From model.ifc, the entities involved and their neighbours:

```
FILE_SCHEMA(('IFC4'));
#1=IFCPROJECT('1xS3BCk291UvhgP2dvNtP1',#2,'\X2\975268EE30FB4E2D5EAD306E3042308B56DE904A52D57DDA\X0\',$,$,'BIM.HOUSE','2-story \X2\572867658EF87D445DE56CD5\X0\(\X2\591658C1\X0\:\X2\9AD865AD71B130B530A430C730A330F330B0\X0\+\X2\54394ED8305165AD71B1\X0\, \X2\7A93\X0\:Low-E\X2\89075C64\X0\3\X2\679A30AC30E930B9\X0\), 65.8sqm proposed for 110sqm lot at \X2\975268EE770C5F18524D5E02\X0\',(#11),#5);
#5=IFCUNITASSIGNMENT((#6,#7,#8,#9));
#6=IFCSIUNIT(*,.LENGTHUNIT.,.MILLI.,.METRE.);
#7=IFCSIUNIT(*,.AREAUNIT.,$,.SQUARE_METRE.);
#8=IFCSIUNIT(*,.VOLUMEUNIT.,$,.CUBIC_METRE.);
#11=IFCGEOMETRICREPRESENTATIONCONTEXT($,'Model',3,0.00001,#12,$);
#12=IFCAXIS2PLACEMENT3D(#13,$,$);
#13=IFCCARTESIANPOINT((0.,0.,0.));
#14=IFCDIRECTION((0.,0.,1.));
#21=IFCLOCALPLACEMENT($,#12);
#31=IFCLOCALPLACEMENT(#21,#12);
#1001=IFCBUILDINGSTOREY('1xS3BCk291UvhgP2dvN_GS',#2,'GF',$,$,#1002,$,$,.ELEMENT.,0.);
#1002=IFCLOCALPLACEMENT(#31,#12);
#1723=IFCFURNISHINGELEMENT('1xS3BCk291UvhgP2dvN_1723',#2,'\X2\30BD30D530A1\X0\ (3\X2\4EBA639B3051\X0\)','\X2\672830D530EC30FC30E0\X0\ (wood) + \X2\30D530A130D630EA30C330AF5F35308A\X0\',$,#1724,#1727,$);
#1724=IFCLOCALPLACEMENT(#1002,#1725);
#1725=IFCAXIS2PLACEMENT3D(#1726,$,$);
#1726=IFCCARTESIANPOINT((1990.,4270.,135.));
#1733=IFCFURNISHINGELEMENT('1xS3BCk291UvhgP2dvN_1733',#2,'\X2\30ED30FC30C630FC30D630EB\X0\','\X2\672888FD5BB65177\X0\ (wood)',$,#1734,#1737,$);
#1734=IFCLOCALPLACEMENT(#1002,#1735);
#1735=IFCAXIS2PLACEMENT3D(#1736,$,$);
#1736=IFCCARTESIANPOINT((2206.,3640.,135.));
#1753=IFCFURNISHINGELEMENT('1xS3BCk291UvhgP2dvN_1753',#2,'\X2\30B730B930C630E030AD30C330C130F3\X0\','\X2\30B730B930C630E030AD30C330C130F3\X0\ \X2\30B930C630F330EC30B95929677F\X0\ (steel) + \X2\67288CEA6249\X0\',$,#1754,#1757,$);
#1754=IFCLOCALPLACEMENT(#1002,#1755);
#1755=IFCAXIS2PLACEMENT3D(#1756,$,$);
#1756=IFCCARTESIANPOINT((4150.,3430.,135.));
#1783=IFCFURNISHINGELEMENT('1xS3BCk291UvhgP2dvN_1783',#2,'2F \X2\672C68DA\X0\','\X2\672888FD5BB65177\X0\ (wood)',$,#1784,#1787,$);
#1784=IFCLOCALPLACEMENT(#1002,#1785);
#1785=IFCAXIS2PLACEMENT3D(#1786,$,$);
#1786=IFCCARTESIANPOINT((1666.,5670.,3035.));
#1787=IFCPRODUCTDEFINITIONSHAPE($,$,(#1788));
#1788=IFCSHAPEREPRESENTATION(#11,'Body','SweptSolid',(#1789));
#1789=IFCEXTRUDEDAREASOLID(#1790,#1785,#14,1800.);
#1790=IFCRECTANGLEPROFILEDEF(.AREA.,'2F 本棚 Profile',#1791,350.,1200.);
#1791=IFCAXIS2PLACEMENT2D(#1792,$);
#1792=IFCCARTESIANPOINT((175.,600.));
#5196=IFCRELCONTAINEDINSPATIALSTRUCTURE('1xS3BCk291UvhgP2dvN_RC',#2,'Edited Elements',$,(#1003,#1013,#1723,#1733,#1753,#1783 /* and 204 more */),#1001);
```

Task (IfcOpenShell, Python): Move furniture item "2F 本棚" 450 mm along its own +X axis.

```python
import ifcopenshell
import ifcopenshell.api.geometry
import ifcopenshell.util.placement
import ifcopenshell.util.unit

model = ifcopenshell.open("model.ifc")
unit_scale = ifcopenshell.util.unit.calculate_unit_scale(model)

item = model.by_id(1783)
matrix = ifcopenshell.util.placement.get_local_placement(item.ObjectPlacement)
matrix[:3, 3] += matrix[:3, 0] * 0.45 / unit_scale
ifcopenshell.api.geometry.edit_object_placement(model, product=item, matrix=matrix, is_si=False)

print(ifcopenshell.util.placement.get_local_placement(item.ObjectPlacement).round(3) + 0.0)

model.write("model_rev.ifc")
```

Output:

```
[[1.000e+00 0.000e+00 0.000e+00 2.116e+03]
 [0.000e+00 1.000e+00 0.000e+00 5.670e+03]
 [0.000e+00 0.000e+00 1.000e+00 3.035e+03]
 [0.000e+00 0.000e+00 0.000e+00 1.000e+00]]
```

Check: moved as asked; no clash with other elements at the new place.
